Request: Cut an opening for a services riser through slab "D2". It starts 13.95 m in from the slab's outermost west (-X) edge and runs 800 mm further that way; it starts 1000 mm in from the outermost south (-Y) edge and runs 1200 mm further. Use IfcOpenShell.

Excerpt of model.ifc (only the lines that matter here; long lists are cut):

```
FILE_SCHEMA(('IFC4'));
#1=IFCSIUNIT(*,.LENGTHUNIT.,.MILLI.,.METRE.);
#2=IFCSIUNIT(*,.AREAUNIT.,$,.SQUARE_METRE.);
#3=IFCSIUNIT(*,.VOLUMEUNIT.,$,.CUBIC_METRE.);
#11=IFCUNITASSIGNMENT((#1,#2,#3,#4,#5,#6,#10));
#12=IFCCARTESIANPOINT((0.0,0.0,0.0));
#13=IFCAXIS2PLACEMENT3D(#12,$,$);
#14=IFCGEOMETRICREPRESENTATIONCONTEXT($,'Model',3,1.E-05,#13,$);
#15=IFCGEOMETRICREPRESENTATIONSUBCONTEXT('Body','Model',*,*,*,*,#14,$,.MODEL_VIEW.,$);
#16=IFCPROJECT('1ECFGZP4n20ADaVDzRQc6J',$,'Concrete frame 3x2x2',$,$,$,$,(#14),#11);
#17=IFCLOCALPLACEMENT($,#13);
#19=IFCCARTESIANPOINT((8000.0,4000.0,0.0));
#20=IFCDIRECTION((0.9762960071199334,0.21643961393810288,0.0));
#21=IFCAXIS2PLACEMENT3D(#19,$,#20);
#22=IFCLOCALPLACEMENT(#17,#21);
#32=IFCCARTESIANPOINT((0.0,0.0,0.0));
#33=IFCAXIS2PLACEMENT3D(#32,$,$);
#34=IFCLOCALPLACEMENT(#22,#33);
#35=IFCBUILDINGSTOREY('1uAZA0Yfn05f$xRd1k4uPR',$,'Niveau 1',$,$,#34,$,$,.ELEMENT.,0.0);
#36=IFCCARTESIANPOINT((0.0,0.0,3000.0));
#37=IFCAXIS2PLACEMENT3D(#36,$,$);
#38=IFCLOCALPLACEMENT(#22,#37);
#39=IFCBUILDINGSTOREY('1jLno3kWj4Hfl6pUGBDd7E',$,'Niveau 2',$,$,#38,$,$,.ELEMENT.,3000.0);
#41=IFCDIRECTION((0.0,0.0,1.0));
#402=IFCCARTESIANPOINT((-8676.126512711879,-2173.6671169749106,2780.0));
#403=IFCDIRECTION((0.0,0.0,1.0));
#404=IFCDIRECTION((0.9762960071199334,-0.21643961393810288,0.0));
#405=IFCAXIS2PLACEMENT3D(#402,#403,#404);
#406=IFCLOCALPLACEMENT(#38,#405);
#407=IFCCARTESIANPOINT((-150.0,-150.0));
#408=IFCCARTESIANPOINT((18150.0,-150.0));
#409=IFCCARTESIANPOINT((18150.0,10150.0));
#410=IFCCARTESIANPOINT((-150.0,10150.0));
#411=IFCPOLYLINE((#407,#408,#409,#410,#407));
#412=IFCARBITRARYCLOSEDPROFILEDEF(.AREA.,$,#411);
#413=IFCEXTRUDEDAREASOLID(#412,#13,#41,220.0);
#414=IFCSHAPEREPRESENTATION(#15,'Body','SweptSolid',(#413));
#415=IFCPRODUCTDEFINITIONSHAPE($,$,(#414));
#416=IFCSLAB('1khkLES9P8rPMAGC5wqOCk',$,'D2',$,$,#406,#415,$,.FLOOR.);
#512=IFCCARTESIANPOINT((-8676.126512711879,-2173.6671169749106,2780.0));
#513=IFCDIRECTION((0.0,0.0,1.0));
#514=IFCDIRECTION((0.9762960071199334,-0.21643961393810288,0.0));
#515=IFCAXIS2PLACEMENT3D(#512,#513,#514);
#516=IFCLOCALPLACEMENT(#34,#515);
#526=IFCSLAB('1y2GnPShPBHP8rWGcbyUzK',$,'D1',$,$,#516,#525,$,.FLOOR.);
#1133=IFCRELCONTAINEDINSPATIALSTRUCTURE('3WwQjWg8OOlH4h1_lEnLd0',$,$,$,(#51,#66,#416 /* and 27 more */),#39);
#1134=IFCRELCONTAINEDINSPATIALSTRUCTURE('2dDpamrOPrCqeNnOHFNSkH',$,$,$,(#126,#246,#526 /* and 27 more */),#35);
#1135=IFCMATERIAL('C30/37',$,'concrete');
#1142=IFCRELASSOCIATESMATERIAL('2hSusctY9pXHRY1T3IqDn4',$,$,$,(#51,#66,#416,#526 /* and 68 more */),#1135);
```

```python
import numpy as np
import ifcopenshell
import ifcopenshell.api.feature
import ifcopenshell.api.geometry
import ifcopenshell.api.root
import ifcopenshell.geom
import ifcopenshell.util.placement
import ifcopenshell.util.representation
import ifcopenshell.util.shape
import ifcopenshell.util.unit

model = ifcopenshell.open("model.ifc")
unit_scale = ifcopenshell.util.unit.calculate_unit_scale(model)
settings = ifcopenshell.geom.settings()


def volume(element):
    """Net volume in cubic metres, openings subtracted."""
    shape = ifcopenshell.geom.create_shape(settings, element)
    return ifcopenshell.util.shape.get_volume(shape.geometry)


slab = model.by_guid("1khkLES9P8rPMAGC5wqOCk")
before = volume(slab)

# Extent in the slab's own axes, in metres. The edges named are its -X and -Y sides.
slab_shape = ifcopenshell.geom.create_shape(settings, slab)
vertices = ifcopenshell.util.shape.get_vertices(slab_shape.geometry)
x_min, y_min, bottom = vertices.min(axis=0)
top = vertices[:, 2].max()

opening = ifcopenshell.api.root.create_entity(model, ifc_class="IfcOpeningElement", name="Services riser opening", predefined_type="OPENING")
context = ifcopenshell.util.representation.get_context(model, "Model", "Body", "MODEL_VIEW")
width, depth = 0.8, 1.2
outline = [(0.0, 0.0), (width, 0.0), (width, depth), (0.0, depth), (0.0, 0.0)]
# Overshoot both faces by 50 mm so the cut is clean.
shape = ifcopenshell.api.geometry.add_slab_representation(
    model, context=context, depth=top - bottom + 0.1, polyline=outline
)
ifcopenshell.api.geometry.assign_representation(model, product=opening, representation=shape)

matrix = ifcopenshell.util.placement.get_local_placement(slab.ObjectPlacement)
matrix[:, 3] = matrix @ np.append(np.array([x_min + 13.95, y_min + 1, bottom - 0.05]) / unit_scale, 1.0)
ifcopenshell.api.geometry.edit_object_placement(model, product=opening, matrix=matrix, is_si=False)
ifcopenshell.api.feature.add_feature(model, feature=opening, element=slab)

after = volume(slab)

print(f"slab volume {before:.3f} -> {after:.3f} m3")

model.write("model-out.ifc")
```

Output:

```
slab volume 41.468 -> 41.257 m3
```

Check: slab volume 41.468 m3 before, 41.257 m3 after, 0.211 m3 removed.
